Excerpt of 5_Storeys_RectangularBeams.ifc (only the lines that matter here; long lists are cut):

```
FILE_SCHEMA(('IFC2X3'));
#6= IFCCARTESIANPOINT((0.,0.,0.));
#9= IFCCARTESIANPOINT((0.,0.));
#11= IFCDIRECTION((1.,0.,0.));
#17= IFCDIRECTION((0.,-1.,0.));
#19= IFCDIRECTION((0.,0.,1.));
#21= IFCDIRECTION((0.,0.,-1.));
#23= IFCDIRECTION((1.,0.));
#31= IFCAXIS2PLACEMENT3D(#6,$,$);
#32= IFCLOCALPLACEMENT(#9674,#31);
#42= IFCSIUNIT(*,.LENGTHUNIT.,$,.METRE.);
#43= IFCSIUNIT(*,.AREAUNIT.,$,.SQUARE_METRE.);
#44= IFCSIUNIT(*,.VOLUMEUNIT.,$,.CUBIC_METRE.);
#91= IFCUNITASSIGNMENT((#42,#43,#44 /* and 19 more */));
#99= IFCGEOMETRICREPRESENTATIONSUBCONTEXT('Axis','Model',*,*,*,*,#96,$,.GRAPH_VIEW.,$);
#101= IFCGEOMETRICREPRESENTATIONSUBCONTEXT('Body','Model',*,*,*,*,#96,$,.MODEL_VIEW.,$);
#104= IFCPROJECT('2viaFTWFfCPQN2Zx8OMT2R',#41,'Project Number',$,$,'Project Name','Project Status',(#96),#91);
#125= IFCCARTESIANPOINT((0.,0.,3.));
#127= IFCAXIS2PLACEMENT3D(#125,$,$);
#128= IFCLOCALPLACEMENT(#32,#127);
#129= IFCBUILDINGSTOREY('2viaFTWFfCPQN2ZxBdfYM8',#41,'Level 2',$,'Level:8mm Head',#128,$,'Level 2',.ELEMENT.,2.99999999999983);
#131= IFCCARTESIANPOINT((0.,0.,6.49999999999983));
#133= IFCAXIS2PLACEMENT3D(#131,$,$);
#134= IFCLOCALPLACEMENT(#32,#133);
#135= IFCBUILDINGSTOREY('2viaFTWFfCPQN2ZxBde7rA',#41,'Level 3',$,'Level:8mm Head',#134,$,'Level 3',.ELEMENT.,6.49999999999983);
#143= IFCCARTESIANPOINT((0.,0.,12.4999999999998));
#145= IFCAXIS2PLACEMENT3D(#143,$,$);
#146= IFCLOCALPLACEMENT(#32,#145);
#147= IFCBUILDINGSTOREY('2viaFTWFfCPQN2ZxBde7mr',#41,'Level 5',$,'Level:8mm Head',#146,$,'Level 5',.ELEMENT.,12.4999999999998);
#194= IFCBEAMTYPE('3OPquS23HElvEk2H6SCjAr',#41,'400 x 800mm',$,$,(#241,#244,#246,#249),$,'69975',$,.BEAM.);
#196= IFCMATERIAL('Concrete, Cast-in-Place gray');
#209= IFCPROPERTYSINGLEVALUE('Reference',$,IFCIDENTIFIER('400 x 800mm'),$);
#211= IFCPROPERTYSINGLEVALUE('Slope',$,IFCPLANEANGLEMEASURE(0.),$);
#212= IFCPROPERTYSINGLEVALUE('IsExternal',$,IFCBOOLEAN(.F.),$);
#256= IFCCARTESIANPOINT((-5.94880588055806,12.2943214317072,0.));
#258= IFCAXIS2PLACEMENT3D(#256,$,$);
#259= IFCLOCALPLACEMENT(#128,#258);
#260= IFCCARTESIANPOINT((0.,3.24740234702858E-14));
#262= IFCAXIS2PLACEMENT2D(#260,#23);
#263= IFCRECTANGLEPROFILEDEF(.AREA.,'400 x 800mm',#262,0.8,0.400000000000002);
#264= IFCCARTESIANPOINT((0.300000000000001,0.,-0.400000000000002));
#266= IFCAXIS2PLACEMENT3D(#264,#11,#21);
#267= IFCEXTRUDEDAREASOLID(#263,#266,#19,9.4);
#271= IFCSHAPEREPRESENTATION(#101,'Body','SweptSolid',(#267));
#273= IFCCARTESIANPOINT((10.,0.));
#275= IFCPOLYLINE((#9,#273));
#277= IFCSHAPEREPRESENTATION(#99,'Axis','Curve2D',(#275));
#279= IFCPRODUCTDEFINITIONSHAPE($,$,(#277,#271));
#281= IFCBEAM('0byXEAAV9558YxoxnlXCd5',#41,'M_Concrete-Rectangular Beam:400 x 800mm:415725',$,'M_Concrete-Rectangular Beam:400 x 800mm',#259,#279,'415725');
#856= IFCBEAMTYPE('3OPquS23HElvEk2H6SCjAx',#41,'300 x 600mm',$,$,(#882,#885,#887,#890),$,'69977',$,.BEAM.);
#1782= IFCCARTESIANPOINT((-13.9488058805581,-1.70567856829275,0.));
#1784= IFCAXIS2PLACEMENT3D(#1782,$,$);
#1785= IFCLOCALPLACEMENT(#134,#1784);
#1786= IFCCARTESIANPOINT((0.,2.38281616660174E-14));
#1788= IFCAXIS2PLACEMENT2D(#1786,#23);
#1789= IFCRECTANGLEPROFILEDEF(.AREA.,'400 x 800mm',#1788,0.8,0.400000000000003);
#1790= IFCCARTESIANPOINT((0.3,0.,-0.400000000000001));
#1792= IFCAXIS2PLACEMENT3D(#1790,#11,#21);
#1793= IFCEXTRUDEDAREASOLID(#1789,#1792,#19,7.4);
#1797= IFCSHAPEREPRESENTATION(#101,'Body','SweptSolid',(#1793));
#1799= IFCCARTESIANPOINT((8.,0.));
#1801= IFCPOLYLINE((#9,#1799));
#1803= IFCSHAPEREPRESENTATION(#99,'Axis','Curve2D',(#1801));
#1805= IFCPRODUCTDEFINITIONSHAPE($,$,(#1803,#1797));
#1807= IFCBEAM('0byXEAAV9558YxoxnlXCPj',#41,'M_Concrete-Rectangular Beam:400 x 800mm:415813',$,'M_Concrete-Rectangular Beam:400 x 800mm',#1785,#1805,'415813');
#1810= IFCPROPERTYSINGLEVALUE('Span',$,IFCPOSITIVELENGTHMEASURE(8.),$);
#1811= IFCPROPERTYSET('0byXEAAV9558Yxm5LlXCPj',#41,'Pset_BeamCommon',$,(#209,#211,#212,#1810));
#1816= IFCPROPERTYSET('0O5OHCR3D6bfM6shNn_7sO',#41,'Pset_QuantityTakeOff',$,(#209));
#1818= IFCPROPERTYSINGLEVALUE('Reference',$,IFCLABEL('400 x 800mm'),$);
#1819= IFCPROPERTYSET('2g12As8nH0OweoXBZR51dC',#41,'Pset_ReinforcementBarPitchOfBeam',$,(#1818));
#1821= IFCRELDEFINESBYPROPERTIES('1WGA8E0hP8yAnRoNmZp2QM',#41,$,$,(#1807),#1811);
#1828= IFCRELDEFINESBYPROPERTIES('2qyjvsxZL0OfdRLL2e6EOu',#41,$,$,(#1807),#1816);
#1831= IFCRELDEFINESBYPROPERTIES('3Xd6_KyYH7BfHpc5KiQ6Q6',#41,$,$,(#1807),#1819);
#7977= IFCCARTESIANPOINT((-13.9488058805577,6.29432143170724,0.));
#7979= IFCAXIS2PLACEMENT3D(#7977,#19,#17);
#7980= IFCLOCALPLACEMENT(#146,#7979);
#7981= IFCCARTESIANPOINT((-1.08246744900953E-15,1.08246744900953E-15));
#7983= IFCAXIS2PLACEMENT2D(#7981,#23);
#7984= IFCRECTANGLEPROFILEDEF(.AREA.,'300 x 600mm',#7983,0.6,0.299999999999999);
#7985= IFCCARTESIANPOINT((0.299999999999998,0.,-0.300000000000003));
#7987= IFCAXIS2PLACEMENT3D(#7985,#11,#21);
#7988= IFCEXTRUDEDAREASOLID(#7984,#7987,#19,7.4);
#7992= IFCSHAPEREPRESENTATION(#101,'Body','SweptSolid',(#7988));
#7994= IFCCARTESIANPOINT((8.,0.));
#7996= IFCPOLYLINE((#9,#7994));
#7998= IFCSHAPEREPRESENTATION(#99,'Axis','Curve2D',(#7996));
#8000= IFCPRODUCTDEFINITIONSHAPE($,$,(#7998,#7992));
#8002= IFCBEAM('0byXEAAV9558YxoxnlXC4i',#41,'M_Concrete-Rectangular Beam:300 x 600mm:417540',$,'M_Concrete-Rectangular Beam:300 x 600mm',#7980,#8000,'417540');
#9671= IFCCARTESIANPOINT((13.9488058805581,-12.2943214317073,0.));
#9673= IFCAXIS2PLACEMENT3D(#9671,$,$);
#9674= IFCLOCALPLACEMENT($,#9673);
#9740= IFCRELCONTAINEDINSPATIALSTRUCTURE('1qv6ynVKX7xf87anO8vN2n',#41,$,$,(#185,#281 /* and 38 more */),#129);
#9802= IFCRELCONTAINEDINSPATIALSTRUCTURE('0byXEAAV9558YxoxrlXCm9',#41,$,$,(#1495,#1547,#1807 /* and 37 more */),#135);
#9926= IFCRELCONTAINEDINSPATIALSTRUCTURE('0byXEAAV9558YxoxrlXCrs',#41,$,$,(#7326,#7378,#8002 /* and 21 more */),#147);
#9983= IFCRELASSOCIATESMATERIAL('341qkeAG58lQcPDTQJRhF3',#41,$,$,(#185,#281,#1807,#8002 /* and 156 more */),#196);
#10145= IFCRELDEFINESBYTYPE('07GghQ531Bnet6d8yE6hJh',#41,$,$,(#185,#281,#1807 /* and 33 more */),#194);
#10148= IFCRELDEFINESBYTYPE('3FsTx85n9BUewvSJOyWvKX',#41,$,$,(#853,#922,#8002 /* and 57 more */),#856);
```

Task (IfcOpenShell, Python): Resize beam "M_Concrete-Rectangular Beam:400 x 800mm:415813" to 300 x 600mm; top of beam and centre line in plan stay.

```python
import ifcopenshell
import ifcopenshell.api.pset
import ifcopenshell.api.type
import ifcopenshell.util.element
import ifcopenshell.util.representation

model = ifcopenshell.open("5_Storeys_RectangularBeams.ifc")

member = model.by_guid("0byXEAAV9558YxoxnlXCPj")
source = next(p for p in model.by_type("IfcRectangleProfileDef") if p.ProfileName == "300 x 600mm")

body = ifcopenshell.util.representation.get_representation(member, "Model", "Body")
solid = body.Items[0]
old_profile = solid.SweptArea

# Copy the section's sizes but keep this member's own profile position.
profile = ifcopenshell.util.element.copy(model, source)
# Profiles are centred, so shift by half the change in depth to hold the top.
shift = (old_profile.XDim - profile.XDim) / 2
x, y = old_profile.Position.Location.Coordinates
up = (-1.0, 0.0)  # upwards, in the solid's own plane
location = model.createIfcCartesianPoint((x + up[0] * shift, y + up[1] * shift))
profile.Position = model.createIfcAxis2Placement2D(location, old_profile.Position.RefDirection)
solid.SweptArea = profile
if not model.get_total_inverses(old_profile):
    ifcopenshell.util.element.remove_deep2(model, old_profile)

new_type = model.by_guid("3OPquS23HElvEk2H6SCjAx")
ifcopenshell.api.type.assign_type(
    model, related_objects=[member], relating_type=new_type, should_map_representations=False
)
member.Name = member.Name.replace("400 x 800mm", "300 x 600mm")
member.ObjectType = "M_Concrete-Rectangular Beam:300 x 600mm"
pset = model.by_id(ifcopenshell.util.element.get_pset(member, "Pset_BeamCommon", should_inherit=False)["id"])
ifcopenshell.api.pset.edit_pset(model, pset=pset, properties={"Reference": "300 x 600mm"})
pset = model.by_id(ifcopenshell.util.element.get_pset(member, "Pset_QuantityTakeOff", should_inherit=False)["id"])
ifcopenshell.api.pset.edit_pset(model, pset=pset, properties={"Reference": "300 x 600mm"})
pset = model.by_id(ifcopenshell.util.element.get_pset(member, "Pset_ReinforcementBarPitchOfBeam", should_inherit=False)["id"])
ifcopenshell.api.pset.edit_pset(model, pset=pset, properties={"Reference": "300 x 600mm"})

print(solid.SweptArea)

model.write("5_Storeys_RectangularBeams_rev.ifc")
```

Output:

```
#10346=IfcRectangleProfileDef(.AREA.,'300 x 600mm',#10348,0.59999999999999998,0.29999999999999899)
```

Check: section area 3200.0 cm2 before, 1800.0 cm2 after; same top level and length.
